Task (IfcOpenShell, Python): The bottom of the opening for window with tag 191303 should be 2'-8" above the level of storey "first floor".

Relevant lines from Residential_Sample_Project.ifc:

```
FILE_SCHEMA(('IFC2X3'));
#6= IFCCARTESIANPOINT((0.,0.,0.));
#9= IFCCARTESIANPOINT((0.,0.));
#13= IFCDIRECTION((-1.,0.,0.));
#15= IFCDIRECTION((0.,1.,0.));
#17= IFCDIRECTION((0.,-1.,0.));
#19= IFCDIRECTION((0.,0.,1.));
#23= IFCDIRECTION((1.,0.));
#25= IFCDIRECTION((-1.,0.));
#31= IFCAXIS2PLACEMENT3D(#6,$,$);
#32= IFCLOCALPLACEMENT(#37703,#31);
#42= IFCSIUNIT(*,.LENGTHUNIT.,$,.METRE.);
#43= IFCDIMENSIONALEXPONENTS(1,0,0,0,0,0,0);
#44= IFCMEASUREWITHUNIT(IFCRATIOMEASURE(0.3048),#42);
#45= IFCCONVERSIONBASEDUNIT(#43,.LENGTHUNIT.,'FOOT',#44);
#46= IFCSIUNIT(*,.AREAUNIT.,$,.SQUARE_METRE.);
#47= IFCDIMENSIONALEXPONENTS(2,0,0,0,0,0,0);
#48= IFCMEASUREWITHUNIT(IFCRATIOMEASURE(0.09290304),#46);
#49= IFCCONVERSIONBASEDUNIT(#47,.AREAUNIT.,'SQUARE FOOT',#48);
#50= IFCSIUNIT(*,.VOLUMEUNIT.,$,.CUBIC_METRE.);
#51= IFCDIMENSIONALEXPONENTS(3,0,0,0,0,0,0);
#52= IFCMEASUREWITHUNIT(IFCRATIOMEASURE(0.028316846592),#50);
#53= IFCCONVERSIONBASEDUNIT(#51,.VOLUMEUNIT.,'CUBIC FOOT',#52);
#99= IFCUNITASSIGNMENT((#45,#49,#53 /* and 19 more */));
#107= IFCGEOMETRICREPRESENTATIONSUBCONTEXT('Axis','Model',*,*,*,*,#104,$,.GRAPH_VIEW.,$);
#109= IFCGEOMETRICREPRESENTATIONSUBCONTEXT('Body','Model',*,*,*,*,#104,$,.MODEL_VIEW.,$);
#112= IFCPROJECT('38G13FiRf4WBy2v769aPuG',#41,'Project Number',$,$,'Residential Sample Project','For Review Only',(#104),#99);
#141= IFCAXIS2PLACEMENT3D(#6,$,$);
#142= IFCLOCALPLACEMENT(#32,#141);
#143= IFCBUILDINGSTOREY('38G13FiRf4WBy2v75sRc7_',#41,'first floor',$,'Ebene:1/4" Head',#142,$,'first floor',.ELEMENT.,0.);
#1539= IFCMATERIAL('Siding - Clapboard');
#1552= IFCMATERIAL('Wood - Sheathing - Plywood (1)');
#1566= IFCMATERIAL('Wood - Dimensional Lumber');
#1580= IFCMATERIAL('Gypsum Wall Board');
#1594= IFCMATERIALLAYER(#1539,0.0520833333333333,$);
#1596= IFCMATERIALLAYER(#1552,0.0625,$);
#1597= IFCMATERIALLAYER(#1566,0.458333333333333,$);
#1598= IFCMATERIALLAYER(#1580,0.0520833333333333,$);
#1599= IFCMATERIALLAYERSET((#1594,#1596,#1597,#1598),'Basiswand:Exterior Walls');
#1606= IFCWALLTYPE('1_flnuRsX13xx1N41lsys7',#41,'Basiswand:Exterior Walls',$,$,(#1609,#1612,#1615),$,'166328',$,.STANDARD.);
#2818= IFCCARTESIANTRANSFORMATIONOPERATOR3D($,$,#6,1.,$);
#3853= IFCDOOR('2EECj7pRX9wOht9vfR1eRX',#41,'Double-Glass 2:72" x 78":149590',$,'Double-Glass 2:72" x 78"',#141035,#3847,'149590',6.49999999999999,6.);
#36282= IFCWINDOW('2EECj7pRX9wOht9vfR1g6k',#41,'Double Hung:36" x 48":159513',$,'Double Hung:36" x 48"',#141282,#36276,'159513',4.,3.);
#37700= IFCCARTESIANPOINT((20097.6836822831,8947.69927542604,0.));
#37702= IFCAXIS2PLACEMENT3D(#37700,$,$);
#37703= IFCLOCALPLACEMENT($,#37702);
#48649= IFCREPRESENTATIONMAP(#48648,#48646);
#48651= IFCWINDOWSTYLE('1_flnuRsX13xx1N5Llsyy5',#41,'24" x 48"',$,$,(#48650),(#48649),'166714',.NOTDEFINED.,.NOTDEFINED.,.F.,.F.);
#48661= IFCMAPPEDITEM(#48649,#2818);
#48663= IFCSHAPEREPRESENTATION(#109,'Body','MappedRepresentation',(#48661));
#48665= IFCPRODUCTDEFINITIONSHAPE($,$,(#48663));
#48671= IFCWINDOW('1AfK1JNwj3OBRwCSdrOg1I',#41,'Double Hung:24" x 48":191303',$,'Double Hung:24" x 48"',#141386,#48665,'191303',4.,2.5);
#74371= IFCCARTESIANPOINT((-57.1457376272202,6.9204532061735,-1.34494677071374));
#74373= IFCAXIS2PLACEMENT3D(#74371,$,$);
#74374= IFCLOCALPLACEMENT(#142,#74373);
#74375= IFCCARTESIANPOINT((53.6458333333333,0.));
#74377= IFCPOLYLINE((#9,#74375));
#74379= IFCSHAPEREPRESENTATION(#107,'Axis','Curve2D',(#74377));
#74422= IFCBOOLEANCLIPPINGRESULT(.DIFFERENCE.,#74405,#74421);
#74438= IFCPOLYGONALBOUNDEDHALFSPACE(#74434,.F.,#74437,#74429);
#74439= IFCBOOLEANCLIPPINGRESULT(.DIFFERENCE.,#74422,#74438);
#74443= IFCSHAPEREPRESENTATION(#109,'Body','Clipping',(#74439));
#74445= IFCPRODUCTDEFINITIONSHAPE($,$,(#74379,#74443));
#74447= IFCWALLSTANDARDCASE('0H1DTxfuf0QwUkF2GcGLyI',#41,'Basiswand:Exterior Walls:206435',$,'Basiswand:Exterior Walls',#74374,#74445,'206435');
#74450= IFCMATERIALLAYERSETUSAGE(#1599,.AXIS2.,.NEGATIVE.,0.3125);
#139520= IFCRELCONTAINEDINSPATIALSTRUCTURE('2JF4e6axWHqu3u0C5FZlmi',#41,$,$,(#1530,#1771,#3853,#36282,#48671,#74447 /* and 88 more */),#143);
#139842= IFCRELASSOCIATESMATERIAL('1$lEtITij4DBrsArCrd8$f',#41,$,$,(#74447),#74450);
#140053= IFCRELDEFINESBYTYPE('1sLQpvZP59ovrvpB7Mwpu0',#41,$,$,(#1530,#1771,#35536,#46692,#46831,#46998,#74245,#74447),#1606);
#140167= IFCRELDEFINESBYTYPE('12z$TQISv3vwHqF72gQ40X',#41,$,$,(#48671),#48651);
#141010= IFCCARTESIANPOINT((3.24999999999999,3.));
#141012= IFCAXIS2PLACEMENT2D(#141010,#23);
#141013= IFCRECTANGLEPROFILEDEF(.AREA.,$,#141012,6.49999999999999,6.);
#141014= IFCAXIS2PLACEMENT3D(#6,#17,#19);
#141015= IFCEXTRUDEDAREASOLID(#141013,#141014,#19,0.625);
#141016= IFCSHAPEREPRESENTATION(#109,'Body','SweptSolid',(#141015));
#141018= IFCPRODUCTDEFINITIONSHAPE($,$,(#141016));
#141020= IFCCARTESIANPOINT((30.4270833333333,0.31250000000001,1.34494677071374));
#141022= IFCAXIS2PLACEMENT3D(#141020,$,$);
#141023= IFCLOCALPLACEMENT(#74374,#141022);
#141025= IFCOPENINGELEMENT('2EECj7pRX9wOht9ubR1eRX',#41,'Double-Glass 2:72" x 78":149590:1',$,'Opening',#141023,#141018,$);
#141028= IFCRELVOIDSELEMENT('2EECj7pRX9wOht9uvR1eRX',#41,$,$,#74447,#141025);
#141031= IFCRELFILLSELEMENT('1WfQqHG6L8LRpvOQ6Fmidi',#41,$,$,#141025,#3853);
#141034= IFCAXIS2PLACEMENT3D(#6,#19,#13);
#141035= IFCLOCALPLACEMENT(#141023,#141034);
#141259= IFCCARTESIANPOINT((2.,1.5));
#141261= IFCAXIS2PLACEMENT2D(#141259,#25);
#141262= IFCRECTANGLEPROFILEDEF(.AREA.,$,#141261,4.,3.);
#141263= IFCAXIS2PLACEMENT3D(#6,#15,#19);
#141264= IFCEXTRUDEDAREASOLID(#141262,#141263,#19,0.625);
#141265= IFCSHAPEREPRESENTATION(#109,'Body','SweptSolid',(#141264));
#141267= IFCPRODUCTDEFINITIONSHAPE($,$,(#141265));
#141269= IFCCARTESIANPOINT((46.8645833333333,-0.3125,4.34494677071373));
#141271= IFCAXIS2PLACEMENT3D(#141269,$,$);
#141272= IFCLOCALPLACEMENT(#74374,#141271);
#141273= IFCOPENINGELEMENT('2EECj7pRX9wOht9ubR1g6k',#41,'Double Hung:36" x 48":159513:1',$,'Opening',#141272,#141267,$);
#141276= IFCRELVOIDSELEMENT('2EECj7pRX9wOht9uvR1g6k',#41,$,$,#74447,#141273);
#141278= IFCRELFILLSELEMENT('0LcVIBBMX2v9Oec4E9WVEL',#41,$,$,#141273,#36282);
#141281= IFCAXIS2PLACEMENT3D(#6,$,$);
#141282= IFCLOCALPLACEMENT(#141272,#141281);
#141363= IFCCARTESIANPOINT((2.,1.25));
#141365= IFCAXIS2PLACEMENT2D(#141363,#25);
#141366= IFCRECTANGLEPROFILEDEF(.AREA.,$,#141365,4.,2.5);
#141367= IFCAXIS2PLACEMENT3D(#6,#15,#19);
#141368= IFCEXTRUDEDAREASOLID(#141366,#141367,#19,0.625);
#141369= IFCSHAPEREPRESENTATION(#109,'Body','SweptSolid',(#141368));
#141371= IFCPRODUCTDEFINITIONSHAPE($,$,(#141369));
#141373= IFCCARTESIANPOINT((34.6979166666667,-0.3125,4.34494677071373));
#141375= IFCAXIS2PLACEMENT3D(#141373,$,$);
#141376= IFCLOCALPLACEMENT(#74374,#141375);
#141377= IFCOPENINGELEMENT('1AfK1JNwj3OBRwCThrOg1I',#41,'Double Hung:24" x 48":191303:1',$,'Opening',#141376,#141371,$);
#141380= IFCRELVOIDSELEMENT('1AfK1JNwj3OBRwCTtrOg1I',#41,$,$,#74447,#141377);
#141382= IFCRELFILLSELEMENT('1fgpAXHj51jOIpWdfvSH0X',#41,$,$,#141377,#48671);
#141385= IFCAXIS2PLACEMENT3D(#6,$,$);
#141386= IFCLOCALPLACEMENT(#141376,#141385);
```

```python
import numpy as np
import ifcopenshell
import ifcopenshell.api.geometry
import ifcopenshell.geom
import ifcopenshell.util.element
import ifcopenshell.util.placement
import ifcopenshell.util.shape
import ifcopenshell.util.unit

model = ifcopenshell.open("Residential_Sample_Project.ifc")
unit_scale = ifcopenshell.util.unit.calculate_unit_scale(model)

window = model.by_guid("1AfK1JNwj3OBRwCSdrOg1I")
opening = window.FillsVoids[0].RelatingOpeningElement
storey = ifcopenshell.util.element.get_container(window, ifc_class="IfcBuildingStorey")
level = ifcopenshell.util.placement.get_local_placement(storey.ObjectPlacement)[2, 3]

# The opening's origin need not be at the sill, so measure its lowest point.
shape = ifcopenshell.geom.create_shape(ifcopenshell.geom.settings(), opening)
bottom = ifcopenshell.util.shape.get_shape_bottom_elevation(shape, shape.geometry) / unit_scale
dz = level + 32 * 0.0254 / unit_scale - bottom

shift = np.array([0.0, 0.0, dz])
# The window is placed relative to its opening, so it follows when the opening moves.
matrix = ifcopenshell.util.placement.get_local_placement(opening.ObjectPlacement)
matrix[:3, 3] += shift
ifcopenshell.api.geometry.edit_object_placement(
    model, product=opening, matrix=matrix, is_si=False, should_transform_children=True
)

print(f"moved by {dz * unit_scale:+.3f} m")

model.write("Residential_Sample_Project_updated.ifc")
```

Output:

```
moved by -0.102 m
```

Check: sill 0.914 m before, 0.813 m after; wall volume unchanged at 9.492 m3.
